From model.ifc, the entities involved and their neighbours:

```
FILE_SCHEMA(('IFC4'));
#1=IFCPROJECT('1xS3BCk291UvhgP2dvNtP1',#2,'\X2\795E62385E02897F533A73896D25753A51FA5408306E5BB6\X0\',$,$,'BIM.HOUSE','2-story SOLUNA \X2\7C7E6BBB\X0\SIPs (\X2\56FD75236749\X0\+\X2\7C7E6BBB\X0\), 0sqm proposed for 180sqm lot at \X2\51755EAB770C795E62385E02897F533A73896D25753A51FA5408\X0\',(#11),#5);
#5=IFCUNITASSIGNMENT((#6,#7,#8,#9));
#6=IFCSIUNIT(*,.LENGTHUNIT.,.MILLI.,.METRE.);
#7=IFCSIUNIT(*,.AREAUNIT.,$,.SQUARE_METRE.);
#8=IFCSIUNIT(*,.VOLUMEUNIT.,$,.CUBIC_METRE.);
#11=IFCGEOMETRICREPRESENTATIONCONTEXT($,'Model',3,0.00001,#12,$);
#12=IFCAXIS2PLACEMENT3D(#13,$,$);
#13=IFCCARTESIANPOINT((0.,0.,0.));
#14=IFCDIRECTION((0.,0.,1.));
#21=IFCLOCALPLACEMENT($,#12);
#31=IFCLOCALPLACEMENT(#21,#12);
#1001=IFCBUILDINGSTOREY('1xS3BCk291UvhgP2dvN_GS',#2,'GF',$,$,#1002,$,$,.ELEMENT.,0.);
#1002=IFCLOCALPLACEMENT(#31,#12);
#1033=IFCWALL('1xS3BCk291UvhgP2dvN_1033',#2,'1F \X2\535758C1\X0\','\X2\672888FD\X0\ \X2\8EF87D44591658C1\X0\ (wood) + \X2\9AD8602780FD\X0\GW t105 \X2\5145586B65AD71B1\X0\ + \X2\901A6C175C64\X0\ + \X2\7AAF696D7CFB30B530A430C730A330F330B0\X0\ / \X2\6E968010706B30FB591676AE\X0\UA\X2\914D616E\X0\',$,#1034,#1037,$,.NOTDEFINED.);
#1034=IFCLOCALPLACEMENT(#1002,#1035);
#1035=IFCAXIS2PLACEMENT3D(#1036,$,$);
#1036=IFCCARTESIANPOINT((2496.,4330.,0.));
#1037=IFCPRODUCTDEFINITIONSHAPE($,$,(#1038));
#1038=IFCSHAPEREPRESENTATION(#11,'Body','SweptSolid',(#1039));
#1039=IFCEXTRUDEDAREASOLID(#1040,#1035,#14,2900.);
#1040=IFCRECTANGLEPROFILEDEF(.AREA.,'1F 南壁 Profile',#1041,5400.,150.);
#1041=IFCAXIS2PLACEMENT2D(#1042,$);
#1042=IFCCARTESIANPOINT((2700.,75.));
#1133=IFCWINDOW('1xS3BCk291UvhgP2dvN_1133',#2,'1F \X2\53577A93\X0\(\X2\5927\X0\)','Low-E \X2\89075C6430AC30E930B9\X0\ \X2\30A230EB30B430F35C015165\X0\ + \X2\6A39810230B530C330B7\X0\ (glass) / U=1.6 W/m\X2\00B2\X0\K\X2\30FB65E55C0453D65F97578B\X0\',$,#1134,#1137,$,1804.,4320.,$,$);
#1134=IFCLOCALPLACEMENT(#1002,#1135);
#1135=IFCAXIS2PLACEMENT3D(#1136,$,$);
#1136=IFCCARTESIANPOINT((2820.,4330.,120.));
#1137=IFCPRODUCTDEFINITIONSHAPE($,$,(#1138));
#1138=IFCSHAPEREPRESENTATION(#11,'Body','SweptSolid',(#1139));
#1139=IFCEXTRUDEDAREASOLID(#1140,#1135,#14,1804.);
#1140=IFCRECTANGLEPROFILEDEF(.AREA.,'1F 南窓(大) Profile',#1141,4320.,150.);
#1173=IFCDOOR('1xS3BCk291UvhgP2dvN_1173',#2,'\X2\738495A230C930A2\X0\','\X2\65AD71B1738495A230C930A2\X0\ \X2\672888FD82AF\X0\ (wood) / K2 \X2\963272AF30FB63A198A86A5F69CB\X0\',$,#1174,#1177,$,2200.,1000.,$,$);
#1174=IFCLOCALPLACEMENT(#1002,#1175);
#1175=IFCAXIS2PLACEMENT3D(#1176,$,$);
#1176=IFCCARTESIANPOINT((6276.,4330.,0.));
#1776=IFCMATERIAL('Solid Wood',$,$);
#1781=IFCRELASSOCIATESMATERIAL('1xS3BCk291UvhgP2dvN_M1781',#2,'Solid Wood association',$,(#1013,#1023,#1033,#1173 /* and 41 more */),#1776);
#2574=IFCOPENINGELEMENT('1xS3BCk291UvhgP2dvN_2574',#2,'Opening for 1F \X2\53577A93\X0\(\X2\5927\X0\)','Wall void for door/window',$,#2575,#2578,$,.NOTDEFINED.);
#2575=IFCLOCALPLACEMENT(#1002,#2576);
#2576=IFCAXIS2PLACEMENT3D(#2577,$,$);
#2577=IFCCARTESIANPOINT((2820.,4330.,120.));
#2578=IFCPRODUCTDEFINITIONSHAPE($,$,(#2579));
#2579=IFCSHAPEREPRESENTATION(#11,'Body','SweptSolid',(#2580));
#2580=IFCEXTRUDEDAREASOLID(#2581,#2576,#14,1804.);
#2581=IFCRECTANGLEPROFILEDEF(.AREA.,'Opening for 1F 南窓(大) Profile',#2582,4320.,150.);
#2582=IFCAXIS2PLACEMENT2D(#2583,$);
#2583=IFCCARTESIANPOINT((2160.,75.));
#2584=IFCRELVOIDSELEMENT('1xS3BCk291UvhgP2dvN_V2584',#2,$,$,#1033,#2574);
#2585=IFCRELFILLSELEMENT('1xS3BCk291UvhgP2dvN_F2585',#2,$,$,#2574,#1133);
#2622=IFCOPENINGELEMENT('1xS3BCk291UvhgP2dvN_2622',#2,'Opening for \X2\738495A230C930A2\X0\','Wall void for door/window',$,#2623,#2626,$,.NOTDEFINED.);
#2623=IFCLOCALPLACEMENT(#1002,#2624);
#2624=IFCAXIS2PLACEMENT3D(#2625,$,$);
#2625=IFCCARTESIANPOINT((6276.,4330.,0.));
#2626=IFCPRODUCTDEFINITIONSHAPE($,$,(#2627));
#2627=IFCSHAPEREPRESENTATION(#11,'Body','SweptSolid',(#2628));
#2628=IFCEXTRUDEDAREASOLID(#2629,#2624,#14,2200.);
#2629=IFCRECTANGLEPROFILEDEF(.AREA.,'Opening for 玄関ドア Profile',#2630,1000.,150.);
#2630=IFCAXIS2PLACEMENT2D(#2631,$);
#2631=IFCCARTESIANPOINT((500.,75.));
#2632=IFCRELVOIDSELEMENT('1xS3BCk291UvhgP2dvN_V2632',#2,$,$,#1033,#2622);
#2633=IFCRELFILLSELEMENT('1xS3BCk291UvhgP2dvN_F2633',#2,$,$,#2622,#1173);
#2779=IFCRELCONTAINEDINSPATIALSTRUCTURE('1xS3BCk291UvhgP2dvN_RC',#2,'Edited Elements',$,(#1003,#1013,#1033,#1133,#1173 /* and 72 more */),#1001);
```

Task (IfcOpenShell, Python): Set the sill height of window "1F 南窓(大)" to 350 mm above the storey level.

```python
import numpy as np
import ifcopenshell
import ifcopenshell.api.geometry
import ifcopenshell.geom
import ifcopenshell.util.element
import ifcopenshell.util.placement
import ifcopenshell.util.shape
import ifcopenshell.util.unit

model = ifcopenshell.open("model.ifc")
unit_scale = ifcopenshell.util.unit.calculate_unit_scale(model)

window = model.by_guid("1xS3BCk291UvhgP2dvN_1133")
opening = window.FillsVoids[0].RelatingOpeningElement
storey = ifcopenshell.util.element.get_container(window, ifc_class="IfcBuildingStorey")
level = ifcopenshell.util.placement.get_local_placement(storey.ObjectPlacement)[2, 3]

# The opening's origin need not be at the sill, so measure its lowest point.
shape = ifcopenshell.geom.create_shape(ifcopenshell.geom.settings(), opening)
bottom = ifcopenshell.util.shape.get_shape_bottom_elevation(shape, shape.geometry) / unit_scale
dz = level + 0.35 / unit_scale - bottom

shift = np.array([0.0, 0.0, dz])
# The window is not placed relative to its opening, so move both.
for product in (opening, window):
    matrix = ifcopenshell.util.placement.get_local_placement(product.ObjectPlacement)
    matrix[:3, 3] += shift
    ifcopenshell.api.geometry.edit_object_placement(model, product=product, matrix=matrix, is_si=False)

print(f"moved by {dz * unit_scale:+.3f} m")

model.write("model-out.ifc")
```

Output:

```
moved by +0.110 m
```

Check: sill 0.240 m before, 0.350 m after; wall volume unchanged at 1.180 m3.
